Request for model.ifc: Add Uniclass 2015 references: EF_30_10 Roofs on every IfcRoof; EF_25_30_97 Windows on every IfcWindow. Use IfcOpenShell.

First a look at what the model holds.

```python
import ifcopenshell

model = ifcopenshell.open("model.ifc")
print(model.schema)
print("classifications:", [c.Name for c in model.by_type("IfcClassification")])
for ifc_class in ("IfcDoor", "IfcRoof", "IfcStair", "IfcWall", "IfcWindow"):
    print(ifc_class, len(model.by_type(ifc_class)))
```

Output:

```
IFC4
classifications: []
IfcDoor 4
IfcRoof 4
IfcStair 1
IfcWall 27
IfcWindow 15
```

```python
import ifcopenshell
import ifcopenshell.api.classification

model = ifcopenshell.open("model.ifc")

system = ifcopenshell.api.classification.add_classification(model, classification="Uniclass 2015")

codes = {
    "IfcRoof": ("EF_30_10", "Roofs"),
    "IfcWindow": ("EF_25_30_97", "Windows"),
}
for ifc_class, (code, name) in codes.items():
    products = model.by_type(ifc_class)
    ifcopenshell.api.classification.add_reference(
        model, products=products, classification=system, identification=code, name=name
    )
    print(code, len(products))

model.write("model_updated.ifc")
```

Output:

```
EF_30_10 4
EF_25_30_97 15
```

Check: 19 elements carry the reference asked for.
